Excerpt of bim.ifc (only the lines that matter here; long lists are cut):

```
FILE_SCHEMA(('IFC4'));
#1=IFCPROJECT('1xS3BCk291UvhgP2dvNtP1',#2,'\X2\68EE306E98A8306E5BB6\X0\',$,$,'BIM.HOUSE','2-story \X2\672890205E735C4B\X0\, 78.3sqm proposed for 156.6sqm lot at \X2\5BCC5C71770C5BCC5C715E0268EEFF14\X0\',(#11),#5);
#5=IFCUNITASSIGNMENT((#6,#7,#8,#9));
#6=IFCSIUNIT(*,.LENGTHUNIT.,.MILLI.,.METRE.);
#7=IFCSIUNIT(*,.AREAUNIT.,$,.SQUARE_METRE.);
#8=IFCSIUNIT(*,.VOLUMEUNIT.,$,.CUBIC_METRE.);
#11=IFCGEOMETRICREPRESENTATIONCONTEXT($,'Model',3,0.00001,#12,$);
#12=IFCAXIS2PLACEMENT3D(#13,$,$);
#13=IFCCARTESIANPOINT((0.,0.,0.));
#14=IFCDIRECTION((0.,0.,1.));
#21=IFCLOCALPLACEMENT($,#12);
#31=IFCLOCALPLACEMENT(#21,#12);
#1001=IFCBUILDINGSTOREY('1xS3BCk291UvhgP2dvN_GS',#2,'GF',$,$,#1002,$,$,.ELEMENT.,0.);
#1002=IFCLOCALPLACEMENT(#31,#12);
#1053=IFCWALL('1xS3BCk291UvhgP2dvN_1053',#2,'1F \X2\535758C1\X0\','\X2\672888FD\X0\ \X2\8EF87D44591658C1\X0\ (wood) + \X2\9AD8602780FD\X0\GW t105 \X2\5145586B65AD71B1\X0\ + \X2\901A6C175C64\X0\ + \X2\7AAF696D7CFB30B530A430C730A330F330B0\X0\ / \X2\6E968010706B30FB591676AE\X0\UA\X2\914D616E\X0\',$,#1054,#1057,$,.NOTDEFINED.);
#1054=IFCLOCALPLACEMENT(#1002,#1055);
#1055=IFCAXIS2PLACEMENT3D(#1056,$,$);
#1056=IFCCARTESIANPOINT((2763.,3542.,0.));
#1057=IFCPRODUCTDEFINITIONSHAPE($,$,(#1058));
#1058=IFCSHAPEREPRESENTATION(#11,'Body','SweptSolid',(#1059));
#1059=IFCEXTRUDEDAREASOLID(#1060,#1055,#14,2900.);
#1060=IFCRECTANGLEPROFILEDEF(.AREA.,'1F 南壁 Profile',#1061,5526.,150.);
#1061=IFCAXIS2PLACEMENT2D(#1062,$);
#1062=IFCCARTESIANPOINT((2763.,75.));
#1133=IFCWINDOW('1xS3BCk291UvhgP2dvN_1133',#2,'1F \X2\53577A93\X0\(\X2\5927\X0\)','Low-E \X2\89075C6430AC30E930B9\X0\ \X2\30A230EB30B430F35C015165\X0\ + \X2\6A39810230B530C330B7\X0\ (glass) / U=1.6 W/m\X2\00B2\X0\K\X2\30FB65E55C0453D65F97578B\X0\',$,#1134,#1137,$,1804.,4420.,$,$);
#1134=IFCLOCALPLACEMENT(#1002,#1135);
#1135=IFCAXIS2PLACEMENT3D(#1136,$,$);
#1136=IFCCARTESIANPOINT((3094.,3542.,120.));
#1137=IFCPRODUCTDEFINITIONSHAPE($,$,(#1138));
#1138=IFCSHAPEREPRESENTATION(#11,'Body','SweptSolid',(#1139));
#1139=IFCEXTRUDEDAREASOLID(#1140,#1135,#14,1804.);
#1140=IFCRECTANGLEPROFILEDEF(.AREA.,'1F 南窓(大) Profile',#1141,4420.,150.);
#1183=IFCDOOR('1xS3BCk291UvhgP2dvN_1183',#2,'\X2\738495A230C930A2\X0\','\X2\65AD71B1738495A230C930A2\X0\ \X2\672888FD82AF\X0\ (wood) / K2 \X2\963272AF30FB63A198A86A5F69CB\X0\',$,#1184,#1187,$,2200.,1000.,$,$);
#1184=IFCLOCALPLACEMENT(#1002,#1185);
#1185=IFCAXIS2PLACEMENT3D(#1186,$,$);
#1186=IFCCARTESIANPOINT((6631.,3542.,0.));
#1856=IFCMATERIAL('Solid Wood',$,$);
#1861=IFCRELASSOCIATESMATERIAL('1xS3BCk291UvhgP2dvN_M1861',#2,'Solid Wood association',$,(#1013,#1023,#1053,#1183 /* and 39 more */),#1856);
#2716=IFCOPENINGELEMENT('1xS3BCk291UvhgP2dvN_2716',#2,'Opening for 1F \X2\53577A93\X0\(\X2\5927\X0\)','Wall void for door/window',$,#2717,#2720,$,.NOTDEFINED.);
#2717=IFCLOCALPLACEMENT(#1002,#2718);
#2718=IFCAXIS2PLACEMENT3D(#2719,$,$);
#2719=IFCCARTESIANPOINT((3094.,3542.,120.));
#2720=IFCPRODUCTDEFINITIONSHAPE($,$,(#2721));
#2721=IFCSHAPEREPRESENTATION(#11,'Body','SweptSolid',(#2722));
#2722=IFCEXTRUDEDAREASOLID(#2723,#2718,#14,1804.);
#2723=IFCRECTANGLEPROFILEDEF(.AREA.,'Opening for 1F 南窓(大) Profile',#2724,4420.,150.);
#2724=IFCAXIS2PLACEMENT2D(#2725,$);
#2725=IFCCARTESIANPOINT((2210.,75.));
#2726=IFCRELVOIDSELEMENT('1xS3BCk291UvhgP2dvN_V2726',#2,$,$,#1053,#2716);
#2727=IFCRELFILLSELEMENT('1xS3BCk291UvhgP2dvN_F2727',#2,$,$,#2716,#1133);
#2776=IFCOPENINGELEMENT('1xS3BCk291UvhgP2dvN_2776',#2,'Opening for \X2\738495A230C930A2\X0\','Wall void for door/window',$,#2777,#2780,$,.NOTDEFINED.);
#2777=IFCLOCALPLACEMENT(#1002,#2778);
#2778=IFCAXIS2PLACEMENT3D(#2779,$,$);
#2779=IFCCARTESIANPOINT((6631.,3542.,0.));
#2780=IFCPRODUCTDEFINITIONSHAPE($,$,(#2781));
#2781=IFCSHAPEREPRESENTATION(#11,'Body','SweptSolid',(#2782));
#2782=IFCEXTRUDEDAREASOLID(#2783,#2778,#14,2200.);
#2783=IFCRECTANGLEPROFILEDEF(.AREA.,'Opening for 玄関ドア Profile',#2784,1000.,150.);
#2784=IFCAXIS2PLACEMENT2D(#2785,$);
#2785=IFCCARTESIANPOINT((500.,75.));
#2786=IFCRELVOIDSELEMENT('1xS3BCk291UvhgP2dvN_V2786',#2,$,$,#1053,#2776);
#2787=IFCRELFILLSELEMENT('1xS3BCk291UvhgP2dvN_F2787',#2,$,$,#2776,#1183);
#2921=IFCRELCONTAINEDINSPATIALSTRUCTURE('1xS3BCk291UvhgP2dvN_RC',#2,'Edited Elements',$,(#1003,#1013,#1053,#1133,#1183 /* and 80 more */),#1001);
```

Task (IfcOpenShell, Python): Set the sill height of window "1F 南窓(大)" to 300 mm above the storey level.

```python
import numpy as np
import ifcopenshell
import ifcopenshell.api.geometry
import ifcopenshell.geom
import ifcopenshell.util.element
import ifcopenshell.util.placement
import ifcopenshell.util.shape
import ifcopenshell.util.unit

model = ifcopenshell.open("bim.ifc")
unit_scale = ifcopenshell.util.unit.calculate_unit_scale(model)

window = model.by_guid("1xS3BCk291UvhgP2dvN_1133")
opening = window.FillsVoids[0].RelatingOpeningElement
storey = ifcopenshell.util.element.get_container(window, ifc_class="IfcBuildingStorey")
level = ifcopenshell.util.placement.get_local_placement(storey.ObjectPlacement)[2, 3]

# The opening's origin need not be at the sill, so measure its lowest point.
shape = ifcopenshell.geom.create_shape(ifcopenshell.geom.settings(), opening)
bottom = ifcopenshell.util.shape.get_shape_bottom_elevation(shape, shape.geometry) / unit_scale
dz = level + 0.3 / unit_scale - bottom

shift = np.array([0.0, 0.0, dz])
# The window is not placed relative to its opening, so move both.
for product in (opening, window):
    matrix = ifcopenshell.util.placement.get_local_placement(product.ObjectPlacement)
    matrix[:3, 3] += shift
    ifcopenshell.api.geometry.edit_object_placement(model, product=product, matrix=matrix, is_si=False)

print(f"moved by {dz * unit_scale:+.3f} m")

model.write("bim-out.ifc")
```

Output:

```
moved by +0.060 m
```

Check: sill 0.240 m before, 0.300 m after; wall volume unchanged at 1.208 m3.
